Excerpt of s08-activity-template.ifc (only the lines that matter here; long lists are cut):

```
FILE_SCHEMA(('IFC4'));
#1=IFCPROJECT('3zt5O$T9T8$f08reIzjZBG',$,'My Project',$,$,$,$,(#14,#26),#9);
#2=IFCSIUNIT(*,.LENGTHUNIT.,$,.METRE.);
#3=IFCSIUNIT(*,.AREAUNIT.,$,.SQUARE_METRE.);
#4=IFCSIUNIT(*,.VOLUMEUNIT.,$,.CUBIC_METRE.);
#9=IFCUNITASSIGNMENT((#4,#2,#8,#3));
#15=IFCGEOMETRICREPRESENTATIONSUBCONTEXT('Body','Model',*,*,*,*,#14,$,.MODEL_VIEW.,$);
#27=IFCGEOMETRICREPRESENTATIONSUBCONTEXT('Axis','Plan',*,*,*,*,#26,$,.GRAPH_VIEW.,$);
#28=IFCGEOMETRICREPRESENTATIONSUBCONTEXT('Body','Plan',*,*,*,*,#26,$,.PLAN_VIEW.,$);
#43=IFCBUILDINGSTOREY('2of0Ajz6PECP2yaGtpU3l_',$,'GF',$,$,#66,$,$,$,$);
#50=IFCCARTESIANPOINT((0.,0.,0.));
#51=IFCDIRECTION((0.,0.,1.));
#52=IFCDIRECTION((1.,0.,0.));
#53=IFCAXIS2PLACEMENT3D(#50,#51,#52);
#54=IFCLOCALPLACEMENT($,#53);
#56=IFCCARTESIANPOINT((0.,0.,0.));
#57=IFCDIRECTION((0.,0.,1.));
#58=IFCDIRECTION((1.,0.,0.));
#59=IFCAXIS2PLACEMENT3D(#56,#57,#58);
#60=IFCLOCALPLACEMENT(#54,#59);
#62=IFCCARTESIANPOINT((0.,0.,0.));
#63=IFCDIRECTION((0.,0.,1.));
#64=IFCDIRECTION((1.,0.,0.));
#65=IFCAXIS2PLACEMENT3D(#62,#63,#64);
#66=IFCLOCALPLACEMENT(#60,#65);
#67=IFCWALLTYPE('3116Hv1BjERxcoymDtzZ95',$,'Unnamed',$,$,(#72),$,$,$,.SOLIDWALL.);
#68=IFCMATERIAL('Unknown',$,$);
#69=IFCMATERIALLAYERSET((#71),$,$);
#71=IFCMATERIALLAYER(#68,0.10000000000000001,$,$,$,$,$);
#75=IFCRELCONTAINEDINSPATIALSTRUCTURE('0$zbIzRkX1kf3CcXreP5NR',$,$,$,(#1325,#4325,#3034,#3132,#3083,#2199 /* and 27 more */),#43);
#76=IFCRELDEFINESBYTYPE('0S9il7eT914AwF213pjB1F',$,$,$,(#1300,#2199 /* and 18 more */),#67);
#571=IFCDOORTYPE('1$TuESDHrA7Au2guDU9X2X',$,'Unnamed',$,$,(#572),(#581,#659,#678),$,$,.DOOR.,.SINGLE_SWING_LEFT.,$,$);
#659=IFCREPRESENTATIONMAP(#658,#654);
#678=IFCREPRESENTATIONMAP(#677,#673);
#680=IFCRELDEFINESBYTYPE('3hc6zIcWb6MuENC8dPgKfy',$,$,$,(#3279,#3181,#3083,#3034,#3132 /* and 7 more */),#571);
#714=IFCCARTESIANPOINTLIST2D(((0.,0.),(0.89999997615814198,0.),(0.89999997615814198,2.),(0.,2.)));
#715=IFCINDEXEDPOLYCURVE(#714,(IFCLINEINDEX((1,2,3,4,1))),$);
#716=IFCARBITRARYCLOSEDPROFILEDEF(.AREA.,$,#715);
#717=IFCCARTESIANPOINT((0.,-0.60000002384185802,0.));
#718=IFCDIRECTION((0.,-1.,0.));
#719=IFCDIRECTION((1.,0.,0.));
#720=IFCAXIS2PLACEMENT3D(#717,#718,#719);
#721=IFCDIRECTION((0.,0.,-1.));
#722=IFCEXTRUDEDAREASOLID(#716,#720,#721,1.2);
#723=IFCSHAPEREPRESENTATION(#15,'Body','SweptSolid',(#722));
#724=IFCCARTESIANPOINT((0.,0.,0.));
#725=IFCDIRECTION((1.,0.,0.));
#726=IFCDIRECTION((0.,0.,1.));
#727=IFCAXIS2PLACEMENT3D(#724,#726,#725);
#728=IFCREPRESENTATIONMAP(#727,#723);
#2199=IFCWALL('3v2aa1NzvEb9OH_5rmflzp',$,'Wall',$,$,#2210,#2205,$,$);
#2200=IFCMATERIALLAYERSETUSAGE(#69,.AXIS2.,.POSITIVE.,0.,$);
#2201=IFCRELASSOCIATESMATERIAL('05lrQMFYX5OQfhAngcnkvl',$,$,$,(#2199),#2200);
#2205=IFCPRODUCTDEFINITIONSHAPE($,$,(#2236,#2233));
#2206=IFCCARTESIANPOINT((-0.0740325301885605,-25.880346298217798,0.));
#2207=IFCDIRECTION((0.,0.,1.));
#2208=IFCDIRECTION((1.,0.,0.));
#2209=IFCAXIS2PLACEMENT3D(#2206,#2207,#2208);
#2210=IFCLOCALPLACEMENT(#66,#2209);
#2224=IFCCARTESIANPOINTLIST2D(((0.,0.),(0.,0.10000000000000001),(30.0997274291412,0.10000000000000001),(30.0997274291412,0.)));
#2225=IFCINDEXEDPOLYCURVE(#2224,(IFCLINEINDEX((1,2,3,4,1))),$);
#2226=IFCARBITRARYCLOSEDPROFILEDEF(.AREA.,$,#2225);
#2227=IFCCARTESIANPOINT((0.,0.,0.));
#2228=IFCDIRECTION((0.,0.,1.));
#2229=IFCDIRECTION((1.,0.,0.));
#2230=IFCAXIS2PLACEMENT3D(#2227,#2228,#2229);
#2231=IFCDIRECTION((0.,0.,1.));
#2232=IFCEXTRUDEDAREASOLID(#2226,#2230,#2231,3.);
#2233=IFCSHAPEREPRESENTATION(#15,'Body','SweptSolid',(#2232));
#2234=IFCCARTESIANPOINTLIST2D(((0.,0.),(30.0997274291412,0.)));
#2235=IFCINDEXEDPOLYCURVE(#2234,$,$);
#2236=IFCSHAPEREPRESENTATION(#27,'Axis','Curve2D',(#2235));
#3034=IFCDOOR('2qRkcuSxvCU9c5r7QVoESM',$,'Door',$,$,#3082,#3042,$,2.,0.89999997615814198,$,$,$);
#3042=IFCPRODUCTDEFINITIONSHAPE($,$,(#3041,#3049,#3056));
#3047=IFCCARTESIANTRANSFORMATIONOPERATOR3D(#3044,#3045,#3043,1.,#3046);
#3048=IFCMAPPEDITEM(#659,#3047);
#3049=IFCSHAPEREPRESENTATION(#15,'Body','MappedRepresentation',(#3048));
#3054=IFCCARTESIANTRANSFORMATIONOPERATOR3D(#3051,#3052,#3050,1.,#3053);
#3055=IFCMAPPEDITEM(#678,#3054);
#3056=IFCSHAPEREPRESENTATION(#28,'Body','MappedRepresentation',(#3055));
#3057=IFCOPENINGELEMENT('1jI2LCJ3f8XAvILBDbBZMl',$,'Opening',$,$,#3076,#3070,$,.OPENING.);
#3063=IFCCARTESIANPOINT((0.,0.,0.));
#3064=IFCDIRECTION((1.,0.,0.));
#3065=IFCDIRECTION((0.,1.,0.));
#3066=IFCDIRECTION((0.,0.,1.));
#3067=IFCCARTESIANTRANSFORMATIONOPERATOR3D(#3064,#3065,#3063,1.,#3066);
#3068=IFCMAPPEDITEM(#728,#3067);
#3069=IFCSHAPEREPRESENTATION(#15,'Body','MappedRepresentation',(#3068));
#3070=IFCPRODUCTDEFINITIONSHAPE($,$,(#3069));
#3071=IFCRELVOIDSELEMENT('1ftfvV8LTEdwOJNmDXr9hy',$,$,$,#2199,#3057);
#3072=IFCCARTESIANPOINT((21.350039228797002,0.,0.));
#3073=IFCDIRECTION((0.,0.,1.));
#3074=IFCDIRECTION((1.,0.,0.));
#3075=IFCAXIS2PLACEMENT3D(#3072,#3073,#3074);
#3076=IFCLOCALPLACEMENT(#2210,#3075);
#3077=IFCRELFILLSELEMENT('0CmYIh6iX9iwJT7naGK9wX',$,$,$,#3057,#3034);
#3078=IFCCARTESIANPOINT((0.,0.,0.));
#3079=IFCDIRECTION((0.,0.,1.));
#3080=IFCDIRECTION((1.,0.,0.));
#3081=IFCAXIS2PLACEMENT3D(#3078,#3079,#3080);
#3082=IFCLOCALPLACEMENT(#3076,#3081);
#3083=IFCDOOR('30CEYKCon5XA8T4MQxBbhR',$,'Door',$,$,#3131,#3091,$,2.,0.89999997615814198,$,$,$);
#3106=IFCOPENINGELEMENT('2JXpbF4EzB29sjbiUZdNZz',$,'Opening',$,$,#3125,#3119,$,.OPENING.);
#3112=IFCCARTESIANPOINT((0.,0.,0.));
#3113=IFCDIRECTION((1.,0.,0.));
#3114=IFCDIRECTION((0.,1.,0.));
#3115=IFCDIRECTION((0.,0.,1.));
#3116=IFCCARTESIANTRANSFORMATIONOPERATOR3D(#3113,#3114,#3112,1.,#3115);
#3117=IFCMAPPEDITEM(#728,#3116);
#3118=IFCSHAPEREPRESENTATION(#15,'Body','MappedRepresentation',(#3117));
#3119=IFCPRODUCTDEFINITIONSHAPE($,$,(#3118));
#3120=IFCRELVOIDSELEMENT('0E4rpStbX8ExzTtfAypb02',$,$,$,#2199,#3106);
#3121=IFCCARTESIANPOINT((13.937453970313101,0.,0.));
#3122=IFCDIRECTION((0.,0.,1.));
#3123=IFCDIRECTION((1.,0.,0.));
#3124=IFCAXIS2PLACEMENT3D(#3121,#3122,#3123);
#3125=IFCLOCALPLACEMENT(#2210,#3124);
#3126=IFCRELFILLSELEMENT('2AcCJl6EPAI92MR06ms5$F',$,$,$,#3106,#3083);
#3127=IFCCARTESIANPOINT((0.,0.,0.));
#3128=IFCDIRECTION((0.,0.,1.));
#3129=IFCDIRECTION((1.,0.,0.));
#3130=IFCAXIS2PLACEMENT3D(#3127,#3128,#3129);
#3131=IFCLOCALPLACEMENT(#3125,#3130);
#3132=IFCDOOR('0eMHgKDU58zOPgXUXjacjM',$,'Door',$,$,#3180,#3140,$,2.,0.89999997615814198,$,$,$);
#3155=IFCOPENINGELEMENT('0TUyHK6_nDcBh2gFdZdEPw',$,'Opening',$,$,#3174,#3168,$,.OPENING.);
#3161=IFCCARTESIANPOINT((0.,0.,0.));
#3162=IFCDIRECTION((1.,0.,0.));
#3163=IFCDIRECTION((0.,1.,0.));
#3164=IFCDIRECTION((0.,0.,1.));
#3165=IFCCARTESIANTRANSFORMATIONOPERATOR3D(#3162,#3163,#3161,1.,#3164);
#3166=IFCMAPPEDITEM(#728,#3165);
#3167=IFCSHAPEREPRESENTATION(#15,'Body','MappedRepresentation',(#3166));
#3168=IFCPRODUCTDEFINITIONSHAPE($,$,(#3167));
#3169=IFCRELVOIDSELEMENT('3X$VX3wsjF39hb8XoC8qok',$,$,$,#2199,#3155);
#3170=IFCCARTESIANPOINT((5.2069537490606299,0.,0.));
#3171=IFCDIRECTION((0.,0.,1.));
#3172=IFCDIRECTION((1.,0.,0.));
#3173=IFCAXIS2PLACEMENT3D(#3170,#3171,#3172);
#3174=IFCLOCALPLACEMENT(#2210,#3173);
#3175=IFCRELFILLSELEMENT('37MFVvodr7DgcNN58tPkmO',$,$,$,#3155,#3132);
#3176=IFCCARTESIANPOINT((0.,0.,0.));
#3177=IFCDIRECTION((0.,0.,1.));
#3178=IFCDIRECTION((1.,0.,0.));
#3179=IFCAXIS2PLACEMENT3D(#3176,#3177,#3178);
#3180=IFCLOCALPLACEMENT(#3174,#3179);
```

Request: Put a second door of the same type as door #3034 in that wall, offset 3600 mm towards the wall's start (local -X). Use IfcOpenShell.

```python
import ifcopenshell
import ifcopenshell.api.feature
import ifcopenshell.api.geometry
import ifcopenshell.api.root
import ifcopenshell.geom
import ifcopenshell.util.element
import ifcopenshell.util.placement
import ifcopenshell.util.shape

model = ifcopenshell.open("s08-activity-template.ifc")
settings = ifcopenshell.geom.settings()


def volume(element):
    """Net volume in cubic metres, openings subtracted."""
    shape = ifcopenshell.geom.create_shape(settings, element)
    return ifcopenshell.util.shape.get_volume(shape.geometry)


door = model.by_guid("2qRkcuSxvCU9c5r7QVoESM")
opening = door.FillsVoids[0].RelatingOpeningElement
wall = opening.VoidsElements[0].RelatingBuildingElement
before = volume(wall)
shift = ifcopenshell.util.placement.get_local_placement(wall.ObjectPlacement)[:3, 0] * -3.6

# copy_class copies the void relationship, type, container and properties, but no geometry.
new_opening = ifcopenshell.api.root.copy_class(model, product=opening)
new_opening.Representation = ifcopenshell.util.element.copy_deep(
    model, opening.Representation, exclude=["IfcGeometricRepresentationContext", "IfcRepresentationMap"]
)
new_door = ifcopenshell.api.root.copy_class(model, product=door)
new_door.Representation = ifcopenshell.util.element.copy_deep(
    model, door.Representation, exclude=["IfcGeometricRepresentationContext", "IfcRepresentationMap"]
)
ifcopenshell.api.feature.add_filling(model, opening=new_opening, element=new_door)

for old, new in ((opening, new_opening), (door, new_door)):
    matrix = ifcopenshell.util.placement.get_local_placement(old.ObjectPlacement)
    matrix[:3, 3] += shift
    ifcopenshell.api.geometry.edit_object_placement(model, product=new, matrix=matrix, is_si=False)

after = volume(wall)

print(f"wall volume {before:.3f} -> {after:.3f} m3")

model.write("s08-activity-template_updated.ifc")
```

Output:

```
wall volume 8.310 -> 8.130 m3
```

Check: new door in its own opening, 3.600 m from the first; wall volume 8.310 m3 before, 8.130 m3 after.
